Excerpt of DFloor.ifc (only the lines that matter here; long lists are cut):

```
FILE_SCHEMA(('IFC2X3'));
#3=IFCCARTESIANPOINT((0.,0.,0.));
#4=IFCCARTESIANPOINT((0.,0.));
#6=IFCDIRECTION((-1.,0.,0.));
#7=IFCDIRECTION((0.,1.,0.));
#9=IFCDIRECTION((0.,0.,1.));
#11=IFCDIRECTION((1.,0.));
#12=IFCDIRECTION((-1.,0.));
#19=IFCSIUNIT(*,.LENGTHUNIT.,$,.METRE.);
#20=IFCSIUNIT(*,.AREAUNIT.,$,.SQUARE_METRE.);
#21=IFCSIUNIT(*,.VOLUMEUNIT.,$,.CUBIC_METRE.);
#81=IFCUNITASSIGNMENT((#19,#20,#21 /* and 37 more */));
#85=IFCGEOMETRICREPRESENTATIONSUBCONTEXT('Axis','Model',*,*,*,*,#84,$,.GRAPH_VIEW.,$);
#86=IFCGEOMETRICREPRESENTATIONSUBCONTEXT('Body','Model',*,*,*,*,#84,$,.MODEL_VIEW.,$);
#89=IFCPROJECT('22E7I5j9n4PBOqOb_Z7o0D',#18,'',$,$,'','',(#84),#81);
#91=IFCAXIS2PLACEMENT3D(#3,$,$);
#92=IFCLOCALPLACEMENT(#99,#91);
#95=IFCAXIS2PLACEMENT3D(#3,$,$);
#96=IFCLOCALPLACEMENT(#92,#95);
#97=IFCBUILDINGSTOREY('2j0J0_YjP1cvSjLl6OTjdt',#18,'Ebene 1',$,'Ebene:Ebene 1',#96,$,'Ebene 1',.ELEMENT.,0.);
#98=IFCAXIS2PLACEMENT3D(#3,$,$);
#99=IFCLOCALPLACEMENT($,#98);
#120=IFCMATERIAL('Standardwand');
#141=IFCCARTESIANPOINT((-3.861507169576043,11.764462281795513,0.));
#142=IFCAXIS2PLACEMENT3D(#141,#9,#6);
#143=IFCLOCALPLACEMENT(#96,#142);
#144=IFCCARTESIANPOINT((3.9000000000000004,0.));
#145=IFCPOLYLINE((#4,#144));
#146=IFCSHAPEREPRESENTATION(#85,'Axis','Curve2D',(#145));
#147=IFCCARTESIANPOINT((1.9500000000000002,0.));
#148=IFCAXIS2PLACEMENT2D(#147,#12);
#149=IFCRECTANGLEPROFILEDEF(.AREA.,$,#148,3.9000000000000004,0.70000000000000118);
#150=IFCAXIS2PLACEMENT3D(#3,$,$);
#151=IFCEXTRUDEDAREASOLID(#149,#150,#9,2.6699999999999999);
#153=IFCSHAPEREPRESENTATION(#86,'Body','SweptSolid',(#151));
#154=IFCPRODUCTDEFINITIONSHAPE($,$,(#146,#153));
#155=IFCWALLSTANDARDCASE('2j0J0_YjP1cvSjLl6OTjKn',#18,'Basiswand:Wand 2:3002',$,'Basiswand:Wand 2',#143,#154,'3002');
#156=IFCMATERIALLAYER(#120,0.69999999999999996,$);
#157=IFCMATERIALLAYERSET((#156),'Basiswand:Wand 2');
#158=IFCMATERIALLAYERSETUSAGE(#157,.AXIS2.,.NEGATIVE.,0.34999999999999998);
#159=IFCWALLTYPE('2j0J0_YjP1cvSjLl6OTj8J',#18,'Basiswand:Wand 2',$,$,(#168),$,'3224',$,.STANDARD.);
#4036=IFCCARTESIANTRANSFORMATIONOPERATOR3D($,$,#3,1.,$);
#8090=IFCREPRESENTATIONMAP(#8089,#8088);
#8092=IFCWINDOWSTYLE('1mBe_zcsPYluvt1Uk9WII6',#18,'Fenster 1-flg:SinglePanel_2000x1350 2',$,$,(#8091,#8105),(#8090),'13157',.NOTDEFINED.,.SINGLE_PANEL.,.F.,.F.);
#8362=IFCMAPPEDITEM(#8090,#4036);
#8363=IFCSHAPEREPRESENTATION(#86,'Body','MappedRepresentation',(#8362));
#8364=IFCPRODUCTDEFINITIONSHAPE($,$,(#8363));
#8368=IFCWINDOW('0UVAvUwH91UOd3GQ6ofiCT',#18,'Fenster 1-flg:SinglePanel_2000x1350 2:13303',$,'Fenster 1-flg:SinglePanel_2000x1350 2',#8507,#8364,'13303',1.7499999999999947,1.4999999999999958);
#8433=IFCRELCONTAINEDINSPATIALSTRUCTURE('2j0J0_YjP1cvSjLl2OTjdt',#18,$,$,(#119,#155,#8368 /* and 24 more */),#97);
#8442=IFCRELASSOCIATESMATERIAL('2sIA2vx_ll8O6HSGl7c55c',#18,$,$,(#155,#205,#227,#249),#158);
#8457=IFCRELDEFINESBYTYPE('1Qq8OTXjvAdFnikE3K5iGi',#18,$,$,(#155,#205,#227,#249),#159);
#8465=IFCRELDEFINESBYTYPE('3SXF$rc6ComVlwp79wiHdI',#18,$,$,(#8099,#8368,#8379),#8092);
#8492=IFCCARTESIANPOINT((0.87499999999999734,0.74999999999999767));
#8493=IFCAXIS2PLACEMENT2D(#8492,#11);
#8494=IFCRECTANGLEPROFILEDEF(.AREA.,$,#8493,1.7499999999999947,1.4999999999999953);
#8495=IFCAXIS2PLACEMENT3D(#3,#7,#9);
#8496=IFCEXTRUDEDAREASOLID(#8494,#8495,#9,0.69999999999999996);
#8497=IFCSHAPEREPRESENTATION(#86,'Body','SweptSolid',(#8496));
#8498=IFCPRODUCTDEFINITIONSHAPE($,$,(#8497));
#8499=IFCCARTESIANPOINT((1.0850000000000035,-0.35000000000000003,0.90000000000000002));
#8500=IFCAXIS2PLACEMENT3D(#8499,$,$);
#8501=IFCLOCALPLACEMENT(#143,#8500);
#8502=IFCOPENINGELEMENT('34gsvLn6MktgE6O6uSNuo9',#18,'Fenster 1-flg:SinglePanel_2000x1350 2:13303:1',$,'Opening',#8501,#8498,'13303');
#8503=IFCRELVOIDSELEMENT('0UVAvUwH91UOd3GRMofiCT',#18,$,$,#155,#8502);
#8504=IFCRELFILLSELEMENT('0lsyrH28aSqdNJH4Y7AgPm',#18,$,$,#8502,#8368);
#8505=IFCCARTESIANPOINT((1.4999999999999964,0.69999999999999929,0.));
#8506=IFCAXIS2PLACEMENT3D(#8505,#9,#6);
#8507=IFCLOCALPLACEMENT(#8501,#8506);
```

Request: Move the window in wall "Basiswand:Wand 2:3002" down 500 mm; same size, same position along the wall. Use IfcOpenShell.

```python
import numpy as np
import ifcopenshell
import ifcopenshell.api.geometry
import ifcopenshell.util.placement
import ifcopenshell.util.unit

model = ifcopenshell.open("DFloor.ifc")
unit_scale = ifcopenshell.util.unit.calculate_unit_scale(model)

window = model.by_guid("0UVAvUwH91UOd3GQ6ofiCT")
opening = window.FillsVoids[0].RelatingOpeningElement
dz = -0.5 / unit_scale

shift = np.array([0.0, 0.0, dz])
# The window is placed relative to its opening, so it follows when the opening moves.
matrix = ifcopenshell.util.placement.get_local_placement(opening.ObjectPlacement)
matrix[:3, 3] += shift
ifcopenshell.api.geometry.edit_object_placement(
    model, product=opening, matrix=matrix, is_si=False, should_transform_children=True
)

print(f"moved by {dz * unit_scale:+.3f} m")

model.write("DFloor_edited.ifc")
```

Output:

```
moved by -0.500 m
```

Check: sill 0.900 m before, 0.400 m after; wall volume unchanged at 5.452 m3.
